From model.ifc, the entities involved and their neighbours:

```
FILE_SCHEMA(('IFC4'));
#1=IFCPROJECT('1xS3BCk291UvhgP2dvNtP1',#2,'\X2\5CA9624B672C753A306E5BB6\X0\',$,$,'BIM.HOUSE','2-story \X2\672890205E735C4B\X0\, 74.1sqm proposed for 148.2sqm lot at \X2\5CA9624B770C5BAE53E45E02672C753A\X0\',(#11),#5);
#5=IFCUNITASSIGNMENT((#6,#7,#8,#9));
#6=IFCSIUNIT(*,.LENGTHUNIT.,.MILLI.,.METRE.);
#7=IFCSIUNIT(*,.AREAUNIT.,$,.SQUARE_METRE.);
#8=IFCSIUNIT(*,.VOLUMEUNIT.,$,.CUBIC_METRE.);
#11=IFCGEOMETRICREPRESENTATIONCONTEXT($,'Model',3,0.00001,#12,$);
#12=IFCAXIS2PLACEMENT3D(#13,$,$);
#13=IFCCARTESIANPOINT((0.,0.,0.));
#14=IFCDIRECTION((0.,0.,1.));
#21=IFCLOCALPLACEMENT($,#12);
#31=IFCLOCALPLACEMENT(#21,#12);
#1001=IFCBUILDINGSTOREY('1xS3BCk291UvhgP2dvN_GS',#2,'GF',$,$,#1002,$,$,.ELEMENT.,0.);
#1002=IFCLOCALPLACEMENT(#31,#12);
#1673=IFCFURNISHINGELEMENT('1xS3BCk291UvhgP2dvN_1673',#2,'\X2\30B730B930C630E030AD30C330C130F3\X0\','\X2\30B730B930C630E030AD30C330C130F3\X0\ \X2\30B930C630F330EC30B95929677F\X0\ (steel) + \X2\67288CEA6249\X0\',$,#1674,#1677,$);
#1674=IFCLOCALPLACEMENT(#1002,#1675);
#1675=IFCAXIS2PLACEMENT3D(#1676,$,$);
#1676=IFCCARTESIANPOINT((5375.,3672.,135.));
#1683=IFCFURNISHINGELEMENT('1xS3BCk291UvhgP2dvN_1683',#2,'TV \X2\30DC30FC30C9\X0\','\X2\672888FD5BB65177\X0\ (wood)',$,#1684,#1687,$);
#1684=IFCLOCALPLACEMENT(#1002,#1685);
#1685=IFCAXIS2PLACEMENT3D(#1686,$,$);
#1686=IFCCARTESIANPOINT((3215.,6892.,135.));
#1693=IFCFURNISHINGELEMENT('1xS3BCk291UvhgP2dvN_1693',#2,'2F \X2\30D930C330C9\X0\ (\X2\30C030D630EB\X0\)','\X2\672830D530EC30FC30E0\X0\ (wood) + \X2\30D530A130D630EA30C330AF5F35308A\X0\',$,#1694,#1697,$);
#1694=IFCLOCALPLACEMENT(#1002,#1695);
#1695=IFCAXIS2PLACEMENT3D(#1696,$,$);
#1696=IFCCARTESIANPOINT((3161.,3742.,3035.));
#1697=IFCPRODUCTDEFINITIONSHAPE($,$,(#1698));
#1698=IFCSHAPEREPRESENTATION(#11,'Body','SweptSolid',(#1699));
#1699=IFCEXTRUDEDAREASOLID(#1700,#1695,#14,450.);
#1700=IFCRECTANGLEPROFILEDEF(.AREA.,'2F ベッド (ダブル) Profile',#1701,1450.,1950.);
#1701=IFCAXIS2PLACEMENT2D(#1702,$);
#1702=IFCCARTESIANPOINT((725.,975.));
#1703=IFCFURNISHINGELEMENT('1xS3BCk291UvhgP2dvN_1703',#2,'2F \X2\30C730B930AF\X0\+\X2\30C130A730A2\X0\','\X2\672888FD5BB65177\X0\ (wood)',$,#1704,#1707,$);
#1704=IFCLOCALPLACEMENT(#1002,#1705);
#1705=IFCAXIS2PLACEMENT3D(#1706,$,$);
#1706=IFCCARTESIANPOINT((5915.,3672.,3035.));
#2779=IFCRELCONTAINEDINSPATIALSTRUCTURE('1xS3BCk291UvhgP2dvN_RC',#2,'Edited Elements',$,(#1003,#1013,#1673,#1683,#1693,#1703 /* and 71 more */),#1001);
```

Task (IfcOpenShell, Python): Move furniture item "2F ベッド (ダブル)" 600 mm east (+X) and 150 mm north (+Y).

```python
import ifcopenshell
import ifcopenshell.api.geometry
import ifcopenshell.util.placement
import ifcopenshell.util.unit

model = ifcopenshell.open("model.ifc")
unit_scale = ifcopenshell.util.unit.calculate_unit_scale(model)

item = model.by_guid("1xS3BCk291UvhgP2dvN_1693")
matrix = ifcopenshell.util.placement.get_local_placement(item.ObjectPlacement)
matrix[0, 3] += 0.6 / unit_scale
matrix[1, 3] += 0.15 / unit_scale
ifcopenshell.api.geometry.edit_object_placement(model, product=item, matrix=matrix, is_si=False)

print(ifcopenshell.util.placement.get_local_placement(item.ObjectPlacement).round(3) + 0.0)

model.write("model_rev.ifc")
```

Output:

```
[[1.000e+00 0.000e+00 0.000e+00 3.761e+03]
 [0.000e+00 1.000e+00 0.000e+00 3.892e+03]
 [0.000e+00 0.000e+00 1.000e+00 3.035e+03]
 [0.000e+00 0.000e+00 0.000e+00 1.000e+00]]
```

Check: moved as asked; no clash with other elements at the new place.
